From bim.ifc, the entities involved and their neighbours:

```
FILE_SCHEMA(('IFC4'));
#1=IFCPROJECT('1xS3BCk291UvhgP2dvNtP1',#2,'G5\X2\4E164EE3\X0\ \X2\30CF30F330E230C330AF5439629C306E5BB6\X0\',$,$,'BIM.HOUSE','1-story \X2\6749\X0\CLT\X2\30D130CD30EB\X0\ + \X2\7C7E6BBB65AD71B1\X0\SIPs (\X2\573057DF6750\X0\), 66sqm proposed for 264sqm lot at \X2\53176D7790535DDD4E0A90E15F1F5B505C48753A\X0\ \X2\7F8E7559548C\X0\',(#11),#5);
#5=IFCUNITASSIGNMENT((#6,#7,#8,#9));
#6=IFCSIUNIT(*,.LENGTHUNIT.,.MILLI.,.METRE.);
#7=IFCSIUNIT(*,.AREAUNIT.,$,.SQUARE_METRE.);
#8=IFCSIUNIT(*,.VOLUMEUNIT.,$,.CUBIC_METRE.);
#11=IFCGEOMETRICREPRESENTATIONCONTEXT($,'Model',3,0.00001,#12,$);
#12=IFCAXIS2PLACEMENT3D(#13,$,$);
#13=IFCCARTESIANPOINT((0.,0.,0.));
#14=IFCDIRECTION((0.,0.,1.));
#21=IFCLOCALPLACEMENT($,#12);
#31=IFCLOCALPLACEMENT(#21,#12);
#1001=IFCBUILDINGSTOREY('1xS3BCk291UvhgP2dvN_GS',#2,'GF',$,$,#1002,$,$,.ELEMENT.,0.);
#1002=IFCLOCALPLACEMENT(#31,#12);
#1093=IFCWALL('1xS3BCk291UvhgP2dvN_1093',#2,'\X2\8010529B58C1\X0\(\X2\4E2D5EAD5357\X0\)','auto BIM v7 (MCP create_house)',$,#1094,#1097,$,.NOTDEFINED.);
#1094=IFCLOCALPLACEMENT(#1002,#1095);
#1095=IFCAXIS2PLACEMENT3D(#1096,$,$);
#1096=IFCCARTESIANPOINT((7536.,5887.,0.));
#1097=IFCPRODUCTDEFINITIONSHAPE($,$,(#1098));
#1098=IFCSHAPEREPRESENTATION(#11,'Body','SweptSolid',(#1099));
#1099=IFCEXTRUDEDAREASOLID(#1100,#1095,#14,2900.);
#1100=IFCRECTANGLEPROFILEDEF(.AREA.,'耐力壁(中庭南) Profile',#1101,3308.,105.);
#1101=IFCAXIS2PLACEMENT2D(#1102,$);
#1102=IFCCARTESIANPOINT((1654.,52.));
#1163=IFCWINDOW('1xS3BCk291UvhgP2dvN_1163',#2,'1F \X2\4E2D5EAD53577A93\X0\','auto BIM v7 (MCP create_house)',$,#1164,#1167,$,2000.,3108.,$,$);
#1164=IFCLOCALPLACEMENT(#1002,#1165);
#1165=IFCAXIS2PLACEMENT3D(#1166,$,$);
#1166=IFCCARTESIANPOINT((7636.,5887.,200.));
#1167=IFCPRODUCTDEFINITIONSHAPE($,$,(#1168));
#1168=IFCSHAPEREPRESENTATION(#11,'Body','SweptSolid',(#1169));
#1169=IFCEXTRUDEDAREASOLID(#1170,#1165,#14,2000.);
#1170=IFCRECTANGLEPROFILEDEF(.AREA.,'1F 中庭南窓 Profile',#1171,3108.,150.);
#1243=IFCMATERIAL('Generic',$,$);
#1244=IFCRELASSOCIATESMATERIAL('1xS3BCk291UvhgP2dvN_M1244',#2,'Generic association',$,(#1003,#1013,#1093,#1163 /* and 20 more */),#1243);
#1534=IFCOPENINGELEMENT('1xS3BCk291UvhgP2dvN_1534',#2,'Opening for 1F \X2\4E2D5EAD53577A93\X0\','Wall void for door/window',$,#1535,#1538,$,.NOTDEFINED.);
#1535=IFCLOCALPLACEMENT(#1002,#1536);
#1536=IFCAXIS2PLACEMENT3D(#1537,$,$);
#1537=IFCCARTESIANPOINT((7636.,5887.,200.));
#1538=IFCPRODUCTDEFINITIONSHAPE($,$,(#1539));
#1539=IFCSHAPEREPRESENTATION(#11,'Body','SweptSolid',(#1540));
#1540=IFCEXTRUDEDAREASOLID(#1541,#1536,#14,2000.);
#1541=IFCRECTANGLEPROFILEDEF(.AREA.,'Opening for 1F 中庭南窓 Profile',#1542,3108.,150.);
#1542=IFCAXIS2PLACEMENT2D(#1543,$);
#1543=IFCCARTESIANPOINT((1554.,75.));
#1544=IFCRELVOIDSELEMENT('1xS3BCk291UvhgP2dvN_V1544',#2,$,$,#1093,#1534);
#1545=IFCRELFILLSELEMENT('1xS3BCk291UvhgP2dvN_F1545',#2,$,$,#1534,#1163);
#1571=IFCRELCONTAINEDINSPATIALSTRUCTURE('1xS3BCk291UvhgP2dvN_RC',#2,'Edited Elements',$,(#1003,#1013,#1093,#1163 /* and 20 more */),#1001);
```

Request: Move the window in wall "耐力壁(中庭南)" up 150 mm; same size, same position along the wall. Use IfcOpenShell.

```python
import numpy as np
import ifcopenshell
import ifcopenshell.api.geometry
import ifcopenshell.util.placement
import ifcopenshell.util.unit

model = ifcopenshell.open("bim.ifc")
unit_scale = ifcopenshell.util.unit.calculate_unit_scale(model)

window = model.by_guid("1xS3BCk291UvhgP2dvN_1163")
opening = window.FillsVoids[0].RelatingOpeningElement
dz = 0.15 / unit_scale

shift = np.array([0.0, 0.0, dz])
# The window is not placed relative to its opening, so move both.
for product in (opening, window):
    matrix = ifcopenshell.util.placement.get_local_placement(product.ObjectPlacement)
    matrix[:3, 3] += shift
    ifcopenshell.api.geometry.edit_object_placement(model, product=product, matrix=matrix, is_si=False)

print(f"moved by {dz * unit_scale:+.3f} m")

model.write("bim_edited.ifc")
```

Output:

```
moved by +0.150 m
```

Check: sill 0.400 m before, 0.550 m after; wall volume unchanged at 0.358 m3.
